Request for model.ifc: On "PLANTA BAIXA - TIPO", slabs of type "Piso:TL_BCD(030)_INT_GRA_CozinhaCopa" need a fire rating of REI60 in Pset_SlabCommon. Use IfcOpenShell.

First a look at what the model holds.

```python
import ifcopenshell
import ifcopenshell.util.element

model = ifcopenshell.open("model.ifc")
print(model.schema)
storey = next(s for s in model.by_type("IfcBuildingStorey") if s.Name == "PLANTA BAIXA - TIPO")
slabs = [e for e in ifcopenshell.util.element.get_decomposition(storey) if e.is_a("IfcSlab")]
seen = {}
for e in slabs:
    element_type = ifcopenshell.util.element.get_type(e)
    key = (element_type.Name if element_type != e and element_type else None, ifcopenshell.util.element.get_pset(e, "Pset_SlabCommon", "FireRating"))
    seen[key] = seen.get(key, 0) + 1
for (name, value), count in sorted(seen.items(), key=str):
    print(count, "x", name, "|", value)
```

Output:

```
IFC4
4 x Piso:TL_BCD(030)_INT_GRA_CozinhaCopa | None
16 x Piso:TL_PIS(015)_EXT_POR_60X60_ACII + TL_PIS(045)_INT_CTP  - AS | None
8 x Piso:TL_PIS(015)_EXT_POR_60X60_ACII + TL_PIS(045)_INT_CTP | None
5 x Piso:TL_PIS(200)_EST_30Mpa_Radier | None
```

```python
import ifcopenshell
import ifcopenshell.api.pset
import ifcopenshell.util.element

model = ifcopenshell.open("model.ifc")

storey = next(s for s in model.by_type("IfcBuildingStorey") if s.Name == "PLANTA BAIXA - TIPO")
slabs = [e for e in ifcopenshell.util.element.get_decomposition(storey) if e.is_a("IfcSlab")]

count = 0
for e in slabs:
    element_type = ifcopenshell.util.element.get_type(e)
    if element_type in (None, e) or element_type.Name != "Piso:TL_BCD(030)_INT_GRA_CozinhaCopa":
        continue
    # add_pset returns the element's existing set when there is one.
    pset = ifcopenshell.api.pset.add_pset(model, product=e, name="Pset_SlabCommon")
    ifcopenshell.api.pset.edit_pset(model, pset=pset, properties={"FireRating": "REI60"})
    count += 1

print(count, "slabs updated")

model.write("model_rev.ifc")
```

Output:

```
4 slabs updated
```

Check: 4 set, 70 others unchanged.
